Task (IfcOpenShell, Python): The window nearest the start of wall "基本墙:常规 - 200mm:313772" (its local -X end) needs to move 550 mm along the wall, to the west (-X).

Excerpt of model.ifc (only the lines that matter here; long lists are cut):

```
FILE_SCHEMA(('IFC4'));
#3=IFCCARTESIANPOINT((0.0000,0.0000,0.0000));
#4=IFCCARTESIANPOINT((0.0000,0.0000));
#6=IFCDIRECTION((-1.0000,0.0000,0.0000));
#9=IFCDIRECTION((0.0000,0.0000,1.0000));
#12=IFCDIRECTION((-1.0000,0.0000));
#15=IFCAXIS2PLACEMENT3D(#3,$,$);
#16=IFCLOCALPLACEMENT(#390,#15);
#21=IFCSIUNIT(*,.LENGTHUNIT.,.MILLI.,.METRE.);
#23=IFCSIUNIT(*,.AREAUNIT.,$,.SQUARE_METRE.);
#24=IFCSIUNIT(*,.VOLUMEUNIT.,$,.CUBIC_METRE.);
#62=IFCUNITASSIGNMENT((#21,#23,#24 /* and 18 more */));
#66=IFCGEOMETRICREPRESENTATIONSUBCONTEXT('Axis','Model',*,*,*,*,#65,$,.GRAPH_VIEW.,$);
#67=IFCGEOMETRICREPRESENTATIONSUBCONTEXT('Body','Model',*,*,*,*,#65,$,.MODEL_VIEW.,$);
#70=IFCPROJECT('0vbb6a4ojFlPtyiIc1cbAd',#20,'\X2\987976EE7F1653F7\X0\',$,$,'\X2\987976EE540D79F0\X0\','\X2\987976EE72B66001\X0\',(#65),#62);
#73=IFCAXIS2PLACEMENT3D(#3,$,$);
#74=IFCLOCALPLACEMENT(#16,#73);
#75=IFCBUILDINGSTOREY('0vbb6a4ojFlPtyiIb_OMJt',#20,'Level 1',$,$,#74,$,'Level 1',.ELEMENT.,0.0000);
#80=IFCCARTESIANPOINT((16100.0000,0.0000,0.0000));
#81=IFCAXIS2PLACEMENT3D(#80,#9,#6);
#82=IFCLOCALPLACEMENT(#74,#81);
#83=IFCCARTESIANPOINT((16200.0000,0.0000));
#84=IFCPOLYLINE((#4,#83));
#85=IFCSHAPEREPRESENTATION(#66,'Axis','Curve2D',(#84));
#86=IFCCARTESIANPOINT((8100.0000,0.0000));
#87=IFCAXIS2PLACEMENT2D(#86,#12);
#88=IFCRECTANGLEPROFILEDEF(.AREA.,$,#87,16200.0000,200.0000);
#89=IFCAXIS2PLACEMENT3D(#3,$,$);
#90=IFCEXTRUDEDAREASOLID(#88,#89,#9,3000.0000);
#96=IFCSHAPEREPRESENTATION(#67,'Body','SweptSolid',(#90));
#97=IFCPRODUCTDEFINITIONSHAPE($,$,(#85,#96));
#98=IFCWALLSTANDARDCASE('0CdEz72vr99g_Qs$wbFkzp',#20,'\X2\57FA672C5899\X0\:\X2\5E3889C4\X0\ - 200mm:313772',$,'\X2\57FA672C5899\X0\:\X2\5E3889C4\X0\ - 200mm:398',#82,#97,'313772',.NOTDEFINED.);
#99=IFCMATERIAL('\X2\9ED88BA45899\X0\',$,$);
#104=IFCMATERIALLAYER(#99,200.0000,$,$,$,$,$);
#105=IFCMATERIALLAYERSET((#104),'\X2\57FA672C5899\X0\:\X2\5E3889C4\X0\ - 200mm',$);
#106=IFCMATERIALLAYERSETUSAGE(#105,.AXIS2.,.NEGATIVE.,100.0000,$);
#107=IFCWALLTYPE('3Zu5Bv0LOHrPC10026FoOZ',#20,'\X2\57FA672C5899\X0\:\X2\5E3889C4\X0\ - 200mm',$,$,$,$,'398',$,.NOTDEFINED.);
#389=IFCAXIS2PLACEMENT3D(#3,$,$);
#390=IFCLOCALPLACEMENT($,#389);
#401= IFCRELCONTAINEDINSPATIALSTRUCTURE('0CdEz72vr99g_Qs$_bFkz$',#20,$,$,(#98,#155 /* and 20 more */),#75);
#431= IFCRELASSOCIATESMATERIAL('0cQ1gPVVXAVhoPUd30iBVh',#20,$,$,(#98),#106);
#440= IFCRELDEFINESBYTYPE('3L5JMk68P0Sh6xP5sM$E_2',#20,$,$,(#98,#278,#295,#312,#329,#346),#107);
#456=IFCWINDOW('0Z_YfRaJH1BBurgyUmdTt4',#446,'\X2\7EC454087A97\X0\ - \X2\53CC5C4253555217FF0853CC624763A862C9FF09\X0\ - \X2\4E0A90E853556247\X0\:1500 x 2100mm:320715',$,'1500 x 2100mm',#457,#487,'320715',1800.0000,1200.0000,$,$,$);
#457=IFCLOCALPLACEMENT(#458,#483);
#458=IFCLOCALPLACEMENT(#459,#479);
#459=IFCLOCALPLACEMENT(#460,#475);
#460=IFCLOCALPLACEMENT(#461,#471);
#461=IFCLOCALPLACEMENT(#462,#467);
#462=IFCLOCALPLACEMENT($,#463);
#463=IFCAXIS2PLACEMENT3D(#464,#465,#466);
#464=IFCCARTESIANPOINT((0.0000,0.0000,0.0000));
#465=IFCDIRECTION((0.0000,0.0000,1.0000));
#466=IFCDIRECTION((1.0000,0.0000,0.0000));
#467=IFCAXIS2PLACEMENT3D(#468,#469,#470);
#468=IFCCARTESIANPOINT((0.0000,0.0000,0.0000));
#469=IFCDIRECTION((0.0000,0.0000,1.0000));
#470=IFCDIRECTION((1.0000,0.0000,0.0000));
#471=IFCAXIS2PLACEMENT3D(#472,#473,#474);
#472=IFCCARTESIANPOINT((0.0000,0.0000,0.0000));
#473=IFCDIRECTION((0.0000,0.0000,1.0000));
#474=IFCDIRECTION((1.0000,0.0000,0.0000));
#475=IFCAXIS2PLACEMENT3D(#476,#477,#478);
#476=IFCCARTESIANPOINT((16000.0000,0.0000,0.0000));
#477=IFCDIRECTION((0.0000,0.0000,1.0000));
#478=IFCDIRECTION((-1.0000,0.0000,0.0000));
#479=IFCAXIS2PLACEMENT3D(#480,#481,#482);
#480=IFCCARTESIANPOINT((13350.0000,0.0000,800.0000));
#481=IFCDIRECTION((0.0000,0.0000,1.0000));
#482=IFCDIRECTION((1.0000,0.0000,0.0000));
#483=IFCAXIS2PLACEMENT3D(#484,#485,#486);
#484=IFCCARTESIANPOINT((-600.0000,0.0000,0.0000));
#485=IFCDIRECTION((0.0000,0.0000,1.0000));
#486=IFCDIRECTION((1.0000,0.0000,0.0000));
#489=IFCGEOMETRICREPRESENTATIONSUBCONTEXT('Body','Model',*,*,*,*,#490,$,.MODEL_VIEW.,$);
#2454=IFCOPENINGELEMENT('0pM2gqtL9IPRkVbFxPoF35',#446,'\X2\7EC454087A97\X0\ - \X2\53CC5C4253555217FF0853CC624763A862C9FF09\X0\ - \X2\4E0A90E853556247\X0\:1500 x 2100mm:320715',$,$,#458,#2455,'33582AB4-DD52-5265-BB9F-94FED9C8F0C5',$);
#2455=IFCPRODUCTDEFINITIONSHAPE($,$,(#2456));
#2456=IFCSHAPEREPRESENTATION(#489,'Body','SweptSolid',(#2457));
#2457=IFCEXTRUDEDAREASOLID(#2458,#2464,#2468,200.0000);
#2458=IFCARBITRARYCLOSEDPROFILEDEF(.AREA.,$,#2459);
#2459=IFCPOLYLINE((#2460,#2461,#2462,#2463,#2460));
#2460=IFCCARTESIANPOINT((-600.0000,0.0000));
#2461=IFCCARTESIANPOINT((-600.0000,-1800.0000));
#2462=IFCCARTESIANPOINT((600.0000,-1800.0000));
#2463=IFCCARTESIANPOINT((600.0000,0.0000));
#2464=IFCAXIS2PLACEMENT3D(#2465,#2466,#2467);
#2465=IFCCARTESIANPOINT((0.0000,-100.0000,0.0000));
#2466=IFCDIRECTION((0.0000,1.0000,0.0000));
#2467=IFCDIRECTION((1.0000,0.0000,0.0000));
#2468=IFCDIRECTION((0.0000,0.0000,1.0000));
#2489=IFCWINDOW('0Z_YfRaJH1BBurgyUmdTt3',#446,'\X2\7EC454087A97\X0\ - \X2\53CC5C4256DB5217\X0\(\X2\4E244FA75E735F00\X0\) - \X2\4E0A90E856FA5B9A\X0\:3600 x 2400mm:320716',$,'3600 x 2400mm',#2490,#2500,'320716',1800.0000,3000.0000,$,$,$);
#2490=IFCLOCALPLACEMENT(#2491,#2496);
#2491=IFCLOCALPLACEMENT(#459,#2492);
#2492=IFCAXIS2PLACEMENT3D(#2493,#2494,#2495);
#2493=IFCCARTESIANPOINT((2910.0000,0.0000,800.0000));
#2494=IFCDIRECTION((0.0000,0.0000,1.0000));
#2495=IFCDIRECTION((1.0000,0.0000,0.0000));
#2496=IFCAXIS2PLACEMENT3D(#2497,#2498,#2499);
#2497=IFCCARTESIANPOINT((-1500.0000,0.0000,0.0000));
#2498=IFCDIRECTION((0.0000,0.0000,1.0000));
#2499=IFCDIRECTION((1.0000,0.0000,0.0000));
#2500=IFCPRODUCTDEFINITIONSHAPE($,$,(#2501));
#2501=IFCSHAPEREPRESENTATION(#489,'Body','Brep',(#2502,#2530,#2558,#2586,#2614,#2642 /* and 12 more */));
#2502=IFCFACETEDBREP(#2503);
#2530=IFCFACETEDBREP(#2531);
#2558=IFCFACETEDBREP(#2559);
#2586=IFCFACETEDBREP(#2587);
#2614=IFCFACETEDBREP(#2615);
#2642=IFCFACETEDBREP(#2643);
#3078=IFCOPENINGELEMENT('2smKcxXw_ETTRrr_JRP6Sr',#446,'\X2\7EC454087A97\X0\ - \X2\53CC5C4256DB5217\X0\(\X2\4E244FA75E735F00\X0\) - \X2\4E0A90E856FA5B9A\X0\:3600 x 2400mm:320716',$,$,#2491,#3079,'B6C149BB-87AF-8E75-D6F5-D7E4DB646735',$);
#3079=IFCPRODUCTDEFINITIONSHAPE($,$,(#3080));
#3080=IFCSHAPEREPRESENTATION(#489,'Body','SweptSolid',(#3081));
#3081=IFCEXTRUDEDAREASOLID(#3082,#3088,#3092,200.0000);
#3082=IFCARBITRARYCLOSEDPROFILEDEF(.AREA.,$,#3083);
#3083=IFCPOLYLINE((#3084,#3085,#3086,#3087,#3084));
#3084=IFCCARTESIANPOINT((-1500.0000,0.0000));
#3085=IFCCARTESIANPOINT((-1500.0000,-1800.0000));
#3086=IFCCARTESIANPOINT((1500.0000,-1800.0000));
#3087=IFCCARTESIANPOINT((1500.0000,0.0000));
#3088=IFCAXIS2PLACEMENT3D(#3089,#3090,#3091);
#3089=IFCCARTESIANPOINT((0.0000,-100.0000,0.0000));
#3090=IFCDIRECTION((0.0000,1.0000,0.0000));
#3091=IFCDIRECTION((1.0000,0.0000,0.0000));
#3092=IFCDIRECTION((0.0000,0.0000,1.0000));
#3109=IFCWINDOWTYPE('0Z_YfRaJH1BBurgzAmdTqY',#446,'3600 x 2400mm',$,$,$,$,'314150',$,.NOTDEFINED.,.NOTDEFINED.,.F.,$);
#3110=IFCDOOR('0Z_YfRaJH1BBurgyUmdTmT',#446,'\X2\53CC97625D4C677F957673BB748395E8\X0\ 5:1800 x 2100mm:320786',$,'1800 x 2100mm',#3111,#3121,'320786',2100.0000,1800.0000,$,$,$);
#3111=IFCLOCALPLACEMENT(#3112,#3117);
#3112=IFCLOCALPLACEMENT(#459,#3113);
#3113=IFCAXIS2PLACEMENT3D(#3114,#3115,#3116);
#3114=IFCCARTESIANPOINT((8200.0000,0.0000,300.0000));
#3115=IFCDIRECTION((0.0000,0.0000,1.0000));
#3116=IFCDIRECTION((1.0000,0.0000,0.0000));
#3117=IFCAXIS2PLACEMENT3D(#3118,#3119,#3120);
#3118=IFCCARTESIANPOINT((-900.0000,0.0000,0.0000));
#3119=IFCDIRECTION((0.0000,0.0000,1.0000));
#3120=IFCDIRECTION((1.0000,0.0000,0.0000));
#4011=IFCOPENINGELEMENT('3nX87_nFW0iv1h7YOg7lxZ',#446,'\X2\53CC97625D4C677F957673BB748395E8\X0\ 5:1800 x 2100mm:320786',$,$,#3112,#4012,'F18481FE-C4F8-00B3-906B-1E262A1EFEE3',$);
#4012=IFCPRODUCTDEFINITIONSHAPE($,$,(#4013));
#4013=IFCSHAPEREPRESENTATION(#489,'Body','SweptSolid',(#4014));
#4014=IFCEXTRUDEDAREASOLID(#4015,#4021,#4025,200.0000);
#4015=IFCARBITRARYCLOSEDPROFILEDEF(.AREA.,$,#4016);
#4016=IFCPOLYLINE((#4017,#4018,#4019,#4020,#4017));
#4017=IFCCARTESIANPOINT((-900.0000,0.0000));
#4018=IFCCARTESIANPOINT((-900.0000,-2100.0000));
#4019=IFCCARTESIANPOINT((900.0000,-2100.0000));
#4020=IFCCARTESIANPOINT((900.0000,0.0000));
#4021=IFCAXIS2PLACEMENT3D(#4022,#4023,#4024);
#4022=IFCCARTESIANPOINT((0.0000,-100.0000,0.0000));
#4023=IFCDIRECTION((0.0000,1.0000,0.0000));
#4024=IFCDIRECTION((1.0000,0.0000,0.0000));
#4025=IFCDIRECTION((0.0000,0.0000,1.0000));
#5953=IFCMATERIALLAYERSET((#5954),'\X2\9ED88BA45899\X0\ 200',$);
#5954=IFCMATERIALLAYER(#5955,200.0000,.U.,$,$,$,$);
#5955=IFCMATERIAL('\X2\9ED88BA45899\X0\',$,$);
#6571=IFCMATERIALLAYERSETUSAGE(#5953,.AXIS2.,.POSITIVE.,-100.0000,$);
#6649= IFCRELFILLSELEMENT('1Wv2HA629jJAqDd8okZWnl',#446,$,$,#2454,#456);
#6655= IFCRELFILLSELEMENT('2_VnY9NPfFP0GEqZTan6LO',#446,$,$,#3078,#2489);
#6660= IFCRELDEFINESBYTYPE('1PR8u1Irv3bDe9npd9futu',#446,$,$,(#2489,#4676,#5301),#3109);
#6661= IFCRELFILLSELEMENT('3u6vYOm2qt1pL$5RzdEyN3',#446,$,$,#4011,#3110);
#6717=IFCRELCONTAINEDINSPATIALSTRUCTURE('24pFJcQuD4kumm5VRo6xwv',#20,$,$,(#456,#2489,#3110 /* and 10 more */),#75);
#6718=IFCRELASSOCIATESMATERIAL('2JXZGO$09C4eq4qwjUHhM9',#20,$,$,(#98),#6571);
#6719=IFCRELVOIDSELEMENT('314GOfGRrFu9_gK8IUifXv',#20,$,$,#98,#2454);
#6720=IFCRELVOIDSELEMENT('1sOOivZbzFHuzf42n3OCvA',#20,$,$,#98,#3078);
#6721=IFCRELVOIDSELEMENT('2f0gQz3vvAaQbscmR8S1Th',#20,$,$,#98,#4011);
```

```python
import ifcopenshell
import ifcopenshell.api.geometry
import ifcopenshell.util.placement
import ifcopenshell.util.unit

model = ifcopenshell.open("model.ifc")
unit_scale = ifcopenshell.util.unit.calculate_unit_scale(model)

window = model.by_guid("0Z_YfRaJH1BBurgyUmdTt3")
opening = window.FillsVoids[0].RelatingOpeningElement
wall = opening.VoidsElements[0].RelatingBuildingElement

wall_matrix = ifcopenshell.util.placement.get_local_placement(wall.ObjectPlacement)
shift = wall_matrix[:3, 0] * 0.55 / unit_scale
before = ifcopenshell.util.placement.get_local_placement(window.ObjectPlacement)[:3, 3].copy()

# The window is placed relative to its opening, so it follows when the opening moves.
matrix = ifcopenshell.util.placement.get_local_placement(opening.ObjectPlacement)
matrix[:3, 3] += shift
ifcopenshell.api.geometry.edit_object_placement(
    model, product=opening, matrix=matrix, is_si=False, should_transform_children=True
)

after = ifcopenshell.util.placement.get_local_placement(window.ObjectPlacement)[:3, 3]
print("window moved by", (after - before).round(3) + 0.0)

model.write("model_updated.ifc")
```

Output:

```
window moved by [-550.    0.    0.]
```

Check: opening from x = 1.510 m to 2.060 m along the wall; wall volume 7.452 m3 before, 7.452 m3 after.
